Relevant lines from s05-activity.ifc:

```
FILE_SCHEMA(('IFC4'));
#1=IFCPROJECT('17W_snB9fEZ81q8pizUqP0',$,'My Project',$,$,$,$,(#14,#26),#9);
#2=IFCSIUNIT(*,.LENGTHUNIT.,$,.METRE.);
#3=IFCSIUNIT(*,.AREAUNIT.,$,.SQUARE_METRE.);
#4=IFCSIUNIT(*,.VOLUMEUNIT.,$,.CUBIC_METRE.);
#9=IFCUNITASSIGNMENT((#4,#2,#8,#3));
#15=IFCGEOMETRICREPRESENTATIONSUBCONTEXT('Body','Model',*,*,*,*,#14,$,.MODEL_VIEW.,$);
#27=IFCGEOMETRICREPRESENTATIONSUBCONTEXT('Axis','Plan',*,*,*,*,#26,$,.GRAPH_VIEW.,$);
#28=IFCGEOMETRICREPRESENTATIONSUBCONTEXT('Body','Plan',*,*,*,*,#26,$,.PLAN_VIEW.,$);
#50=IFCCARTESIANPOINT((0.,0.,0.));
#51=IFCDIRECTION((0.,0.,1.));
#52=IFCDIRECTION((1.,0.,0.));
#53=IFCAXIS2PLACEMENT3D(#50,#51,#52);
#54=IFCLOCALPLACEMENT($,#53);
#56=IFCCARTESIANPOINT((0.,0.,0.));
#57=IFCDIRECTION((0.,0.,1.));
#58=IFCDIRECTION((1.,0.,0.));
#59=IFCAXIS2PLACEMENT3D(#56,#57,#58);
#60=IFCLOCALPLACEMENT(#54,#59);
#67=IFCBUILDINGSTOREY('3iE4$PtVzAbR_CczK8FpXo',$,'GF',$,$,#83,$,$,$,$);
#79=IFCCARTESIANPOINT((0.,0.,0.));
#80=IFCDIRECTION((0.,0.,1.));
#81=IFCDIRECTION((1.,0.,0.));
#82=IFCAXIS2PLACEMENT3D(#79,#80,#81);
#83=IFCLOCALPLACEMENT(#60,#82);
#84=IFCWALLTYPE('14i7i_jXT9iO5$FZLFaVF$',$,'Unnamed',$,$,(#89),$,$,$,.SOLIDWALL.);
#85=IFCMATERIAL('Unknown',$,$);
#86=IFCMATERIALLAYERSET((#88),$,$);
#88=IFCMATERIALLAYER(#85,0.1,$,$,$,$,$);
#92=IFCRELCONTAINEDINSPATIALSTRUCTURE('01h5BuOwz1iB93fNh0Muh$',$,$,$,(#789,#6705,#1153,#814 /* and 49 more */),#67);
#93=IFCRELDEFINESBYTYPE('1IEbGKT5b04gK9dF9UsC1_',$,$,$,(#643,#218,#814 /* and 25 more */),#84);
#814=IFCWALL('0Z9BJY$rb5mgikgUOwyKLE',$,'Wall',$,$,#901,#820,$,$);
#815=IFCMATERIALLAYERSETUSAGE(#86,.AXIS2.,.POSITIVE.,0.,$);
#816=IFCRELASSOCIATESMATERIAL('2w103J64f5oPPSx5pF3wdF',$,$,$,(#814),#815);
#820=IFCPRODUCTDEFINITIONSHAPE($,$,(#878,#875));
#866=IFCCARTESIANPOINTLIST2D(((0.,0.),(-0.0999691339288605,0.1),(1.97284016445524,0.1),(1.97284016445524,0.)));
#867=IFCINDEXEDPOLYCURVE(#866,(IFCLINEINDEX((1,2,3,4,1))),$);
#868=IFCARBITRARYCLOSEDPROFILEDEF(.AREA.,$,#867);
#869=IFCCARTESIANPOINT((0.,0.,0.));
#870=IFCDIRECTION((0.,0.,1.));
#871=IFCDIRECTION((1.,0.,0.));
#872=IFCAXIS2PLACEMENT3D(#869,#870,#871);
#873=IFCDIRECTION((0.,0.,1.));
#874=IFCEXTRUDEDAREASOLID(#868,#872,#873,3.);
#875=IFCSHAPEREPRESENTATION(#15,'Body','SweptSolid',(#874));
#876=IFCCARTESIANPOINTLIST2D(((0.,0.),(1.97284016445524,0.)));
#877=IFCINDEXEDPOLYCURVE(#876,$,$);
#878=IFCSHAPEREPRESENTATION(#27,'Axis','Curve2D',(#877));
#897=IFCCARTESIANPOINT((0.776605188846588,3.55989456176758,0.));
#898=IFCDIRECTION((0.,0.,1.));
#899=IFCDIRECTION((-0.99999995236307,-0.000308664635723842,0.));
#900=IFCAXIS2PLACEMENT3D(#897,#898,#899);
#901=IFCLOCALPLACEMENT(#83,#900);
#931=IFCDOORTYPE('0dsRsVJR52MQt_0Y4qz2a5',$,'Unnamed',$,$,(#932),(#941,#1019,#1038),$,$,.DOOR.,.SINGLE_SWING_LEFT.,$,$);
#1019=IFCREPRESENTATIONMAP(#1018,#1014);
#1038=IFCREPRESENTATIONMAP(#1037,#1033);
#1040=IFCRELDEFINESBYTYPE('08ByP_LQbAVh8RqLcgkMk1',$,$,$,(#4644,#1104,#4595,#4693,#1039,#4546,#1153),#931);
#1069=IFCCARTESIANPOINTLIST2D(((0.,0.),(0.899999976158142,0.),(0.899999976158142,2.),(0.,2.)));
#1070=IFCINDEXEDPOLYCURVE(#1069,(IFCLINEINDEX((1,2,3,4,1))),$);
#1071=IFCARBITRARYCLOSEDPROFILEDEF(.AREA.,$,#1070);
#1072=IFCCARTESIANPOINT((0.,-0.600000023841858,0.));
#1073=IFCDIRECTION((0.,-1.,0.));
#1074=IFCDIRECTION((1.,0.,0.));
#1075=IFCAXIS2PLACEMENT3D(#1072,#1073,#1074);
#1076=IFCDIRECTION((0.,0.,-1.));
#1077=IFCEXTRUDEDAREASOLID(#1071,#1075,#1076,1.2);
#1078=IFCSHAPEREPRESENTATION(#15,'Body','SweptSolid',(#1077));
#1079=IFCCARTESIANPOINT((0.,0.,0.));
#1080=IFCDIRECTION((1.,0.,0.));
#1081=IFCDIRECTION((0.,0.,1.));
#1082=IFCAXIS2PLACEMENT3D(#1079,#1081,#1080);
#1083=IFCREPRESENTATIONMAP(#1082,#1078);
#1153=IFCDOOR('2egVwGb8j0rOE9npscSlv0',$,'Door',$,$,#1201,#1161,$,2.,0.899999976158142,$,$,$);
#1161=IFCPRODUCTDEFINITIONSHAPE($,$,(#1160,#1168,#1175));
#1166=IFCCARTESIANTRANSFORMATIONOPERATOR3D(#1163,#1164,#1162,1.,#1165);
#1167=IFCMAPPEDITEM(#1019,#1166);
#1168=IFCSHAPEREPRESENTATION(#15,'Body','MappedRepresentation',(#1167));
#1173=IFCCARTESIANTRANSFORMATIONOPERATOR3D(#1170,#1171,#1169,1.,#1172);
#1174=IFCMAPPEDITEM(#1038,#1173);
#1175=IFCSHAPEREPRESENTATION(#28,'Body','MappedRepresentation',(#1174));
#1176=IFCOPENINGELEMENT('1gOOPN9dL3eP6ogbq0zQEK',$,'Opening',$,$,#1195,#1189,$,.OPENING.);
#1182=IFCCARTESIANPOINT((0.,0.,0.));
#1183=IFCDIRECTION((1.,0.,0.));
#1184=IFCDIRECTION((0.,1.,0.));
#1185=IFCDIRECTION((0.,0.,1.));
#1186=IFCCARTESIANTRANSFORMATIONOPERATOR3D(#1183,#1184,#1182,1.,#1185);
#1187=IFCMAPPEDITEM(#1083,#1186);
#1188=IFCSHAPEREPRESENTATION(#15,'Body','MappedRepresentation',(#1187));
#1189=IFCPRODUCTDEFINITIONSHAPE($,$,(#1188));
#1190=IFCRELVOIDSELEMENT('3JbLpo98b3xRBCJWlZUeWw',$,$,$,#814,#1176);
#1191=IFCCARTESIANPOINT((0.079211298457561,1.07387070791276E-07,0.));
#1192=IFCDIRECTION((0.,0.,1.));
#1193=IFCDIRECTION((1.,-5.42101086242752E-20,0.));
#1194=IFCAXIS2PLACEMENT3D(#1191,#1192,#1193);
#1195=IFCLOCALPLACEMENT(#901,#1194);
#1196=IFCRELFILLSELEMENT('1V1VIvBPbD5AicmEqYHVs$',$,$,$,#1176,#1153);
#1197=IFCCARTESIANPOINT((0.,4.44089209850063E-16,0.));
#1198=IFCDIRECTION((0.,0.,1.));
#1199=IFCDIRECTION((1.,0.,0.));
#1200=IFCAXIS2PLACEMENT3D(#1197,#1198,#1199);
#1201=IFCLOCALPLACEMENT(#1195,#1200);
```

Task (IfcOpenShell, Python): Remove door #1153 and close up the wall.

```python
import ifcopenshell
import ifcopenshell.api.feature
import ifcopenshell.api.root
import ifcopenshell.geom
import ifcopenshell.util.shape

model = ifcopenshell.open("s05-activity.ifc")
settings = ifcopenshell.geom.settings()


def volume(element):
    """Net volume in cubic metres, openings subtracted."""
    shape = ifcopenshell.geom.create_shape(settings, element)
    return ifcopenshell.util.shape.get_volume(shape.geometry)


door = model.by_id(1153)
opening = door.FillsVoids[0].RelatingOpeningElement
wall = opening.VoidsElements[0].RelatingBuildingElement
before = volume(wall)

ifcopenshell.api.root.remove_product(model, product=door)
ifcopenshell.api.feature.remove_feature(model, feature=opening)

after = volume(wall)

print(f"wall volume {before:.3f} -> {after:.3f} m3")

model.write("s05-activity-out.ifc")
```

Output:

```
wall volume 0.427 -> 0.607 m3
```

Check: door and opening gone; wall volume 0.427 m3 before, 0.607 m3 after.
